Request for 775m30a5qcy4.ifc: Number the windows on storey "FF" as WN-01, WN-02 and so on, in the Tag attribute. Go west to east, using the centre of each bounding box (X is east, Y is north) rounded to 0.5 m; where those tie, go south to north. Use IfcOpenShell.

First a look at what the model holds.

```python
import ifcopenshell
import ifcopenshell.util.element
import ifcopenshell.util.placement

model = ifcopenshell.open("775m30a5qcy4.ifc")
print(model.schema)
storey = next(s for s in model.by_type("IfcBuildingStorey") if s.Name == "FF")
windows = [e for e in ifcopenshell.util.element.get_decomposition(storey) if e.is_a("IfcWindow")]
for e in sorted(windows, key=lambda e: e.id()):
    origin = ifcopenshell.util.placement.get_local_placement(e.ObjectPlacement)[:3, 3]
    print(e.id(), e.Tag, e.Name, origin.round(2) + 0.0, sep=" | ")
```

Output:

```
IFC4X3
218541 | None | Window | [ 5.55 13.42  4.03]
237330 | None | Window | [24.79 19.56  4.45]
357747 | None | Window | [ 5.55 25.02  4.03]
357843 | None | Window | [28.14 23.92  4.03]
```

```python
import ifcopenshell
import ifcopenshell.geom
import ifcopenshell.util.element
import ifcopenshell.util.shape

model = ifcopenshell.open("775m30a5qcy4.ifc")
settings = ifcopenshell.geom.settings()
settings.set("use-world-coords", True)


def centre(element):
    shape = ifcopenshell.geom.create_shape(settings, element)
    return ifcopenshell.util.shape.get_bbox_centroid(shape.geometry)


storey = next(s for s in model.by_type("IfcBuildingStorey") if s.Name == "FF")
windows = [e for e in ifcopenshell.util.element.get_decomposition(storey) if e.is_a("IfcWindow")]

# Insertion points can sit at a corner or the storey origin, so sort by the geometry (in metres).
centres = {e: centre(e) for e in windows}
windows.sort(key=lambda e: (round(centres[e][0] / 0.5), centres[e][1]))

for i, e in enumerate(windows, start=1):
    number = f"WN-{i:02d}"
    e.Tag = number
    print(e.id(), number)

model.write("775m30a5qcy4-out.ifc")
```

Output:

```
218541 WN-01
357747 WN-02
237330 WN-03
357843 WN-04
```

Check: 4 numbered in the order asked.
